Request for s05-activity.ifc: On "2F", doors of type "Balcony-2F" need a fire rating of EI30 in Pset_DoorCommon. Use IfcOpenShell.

First a look at what the model holds.

```python
import ifcopenshell
import ifcopenshell.util.element

model = ifcopenshell.open("s05-activity.ifc")
print(model.schema)
storey = next(s for s in model.by_type("IfcBuildingStorey") if s.Name == "2F")
doors = [e for e in ifcopenshell.util.element.get_decomposition(storey) if e.is_a("IfcDoor")]
seen = {}
for e in doors:
    element_type = ifcopenshell.util.element.get_type(e)
    key = (element_type.Name if element_type != e and element_type else None, ifcopenshell.util.element.get_pset(e, "Pset_DoorCommon", "FireRating"))
    seen[key] = seen.get(key, 0) + 1
for (name, value), count in sorted(seen.items(), key=str):
    print(count, "x", name, "|", value)
```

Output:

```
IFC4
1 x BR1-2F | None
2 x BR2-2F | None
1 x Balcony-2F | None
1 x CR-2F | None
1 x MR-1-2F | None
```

```python
import ifcopenshell
import ifcopenshell.api.pset
import ifcopenshell.util.element

model = ifcopenshell.open("s05-activity.ifc")

storey = next(s for s in model.by_type("IfcBuildingStorey") if s.Name == "2F")
doors = [e for e in ifcopenshell.util.element.get_decomposition(storey) if e.is_a("IfcDoor")]

count = 0
for e in doors:
    element_type = ifcopenshell.util.element.get_type(e)
    if element_type in (None, e) or element_type.Name != "Balcony-2F":
        continue
    # add_pset returns the element's existing set when there is one.
    pset = ifcopenshell.api.pset.add_pset(model, product=e, name="Pset_DoorCommon")
    ifcopenshell.api.pset.edit_pset(model, pset=pset, properties={"FireRating": "EI30"})
    count += 1

print(count, "doors updated")

model.write("s05-activity_updated.ifc")
```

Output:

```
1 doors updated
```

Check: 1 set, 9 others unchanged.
